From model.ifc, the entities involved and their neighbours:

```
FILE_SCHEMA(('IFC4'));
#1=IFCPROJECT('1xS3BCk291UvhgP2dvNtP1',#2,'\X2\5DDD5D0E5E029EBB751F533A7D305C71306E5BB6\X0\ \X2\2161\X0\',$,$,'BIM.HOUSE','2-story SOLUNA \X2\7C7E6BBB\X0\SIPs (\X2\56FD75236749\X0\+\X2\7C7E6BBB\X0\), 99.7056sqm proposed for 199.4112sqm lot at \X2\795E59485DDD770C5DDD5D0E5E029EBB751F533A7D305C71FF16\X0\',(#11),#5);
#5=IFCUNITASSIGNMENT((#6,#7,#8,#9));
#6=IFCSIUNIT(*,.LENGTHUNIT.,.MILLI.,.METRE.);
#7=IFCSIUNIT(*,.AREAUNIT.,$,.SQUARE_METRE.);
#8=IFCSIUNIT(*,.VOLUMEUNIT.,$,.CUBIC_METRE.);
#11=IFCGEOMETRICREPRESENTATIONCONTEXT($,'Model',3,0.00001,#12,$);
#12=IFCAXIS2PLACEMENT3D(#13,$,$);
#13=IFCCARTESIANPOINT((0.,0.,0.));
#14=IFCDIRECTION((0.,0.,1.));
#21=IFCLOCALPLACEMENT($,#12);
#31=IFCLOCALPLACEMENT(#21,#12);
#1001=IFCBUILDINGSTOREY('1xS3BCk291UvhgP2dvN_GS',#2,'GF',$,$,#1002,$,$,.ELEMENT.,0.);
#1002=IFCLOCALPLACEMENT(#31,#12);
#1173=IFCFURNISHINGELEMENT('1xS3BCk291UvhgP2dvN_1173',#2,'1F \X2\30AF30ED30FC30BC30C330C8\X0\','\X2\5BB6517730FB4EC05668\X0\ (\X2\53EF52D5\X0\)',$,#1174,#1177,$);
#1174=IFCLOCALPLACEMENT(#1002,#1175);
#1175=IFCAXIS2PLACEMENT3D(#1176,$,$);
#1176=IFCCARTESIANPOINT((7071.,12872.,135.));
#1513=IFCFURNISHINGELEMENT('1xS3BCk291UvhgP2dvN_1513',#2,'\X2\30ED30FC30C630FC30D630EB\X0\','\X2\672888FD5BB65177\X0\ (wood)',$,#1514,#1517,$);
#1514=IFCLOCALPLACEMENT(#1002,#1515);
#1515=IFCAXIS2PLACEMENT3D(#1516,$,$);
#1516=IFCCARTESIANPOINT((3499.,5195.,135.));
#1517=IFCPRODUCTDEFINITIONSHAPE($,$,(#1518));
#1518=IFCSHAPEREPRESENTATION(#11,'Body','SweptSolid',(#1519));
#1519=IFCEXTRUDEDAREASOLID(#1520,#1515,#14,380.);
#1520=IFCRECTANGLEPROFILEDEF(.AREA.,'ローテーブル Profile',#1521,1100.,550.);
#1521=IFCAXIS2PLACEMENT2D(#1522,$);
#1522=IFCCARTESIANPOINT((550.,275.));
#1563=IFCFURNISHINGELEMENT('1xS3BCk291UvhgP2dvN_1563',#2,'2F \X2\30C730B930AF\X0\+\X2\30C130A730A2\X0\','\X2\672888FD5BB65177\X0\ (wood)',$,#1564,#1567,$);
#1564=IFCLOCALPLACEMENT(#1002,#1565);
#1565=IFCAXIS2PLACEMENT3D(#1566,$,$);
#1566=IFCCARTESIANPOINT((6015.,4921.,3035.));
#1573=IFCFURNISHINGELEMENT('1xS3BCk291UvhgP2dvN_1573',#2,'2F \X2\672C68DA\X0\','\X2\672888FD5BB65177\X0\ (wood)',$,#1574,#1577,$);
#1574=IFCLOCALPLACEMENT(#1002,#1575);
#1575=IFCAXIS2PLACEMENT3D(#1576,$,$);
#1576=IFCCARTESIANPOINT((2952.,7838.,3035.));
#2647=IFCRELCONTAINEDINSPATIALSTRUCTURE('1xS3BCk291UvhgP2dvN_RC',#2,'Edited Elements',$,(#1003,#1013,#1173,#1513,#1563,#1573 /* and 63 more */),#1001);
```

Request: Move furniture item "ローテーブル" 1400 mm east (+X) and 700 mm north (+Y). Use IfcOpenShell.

```python
import ifcopenshell
import ifcopenshell.api.geometry
import ifcopenshell.util.placement
import ifcopenshell.util.unit

model = ifcopenshell.open("model.ifc")
unit_scale = ifcopenshell.util.unit.calculate_unit_scale(model)

item = model.by_guid("1xS3BCk291UvhgP2dvN_1513")
matrix = ifcopenshell.util.placement.get_local_placement(item.ObjectPlacement)
matrix[0, 3] += 1.4 / unit_scale
matrix[1, 3] += 0.7 / unit_scale
ifcopenshell.api.geometry.edit_object_placement(model, product=item, matrix=matrix, is_si=False)

print(ifcopenshell.util.placement.get_local_placement(item.ObjectPlacement).round(3) + 0.0)

model.write("model-out.ifc")
```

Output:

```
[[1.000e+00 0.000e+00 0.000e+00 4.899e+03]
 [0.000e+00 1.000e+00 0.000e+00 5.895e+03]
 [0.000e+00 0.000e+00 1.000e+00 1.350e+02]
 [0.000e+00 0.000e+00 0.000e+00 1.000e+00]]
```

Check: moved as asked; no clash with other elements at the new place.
